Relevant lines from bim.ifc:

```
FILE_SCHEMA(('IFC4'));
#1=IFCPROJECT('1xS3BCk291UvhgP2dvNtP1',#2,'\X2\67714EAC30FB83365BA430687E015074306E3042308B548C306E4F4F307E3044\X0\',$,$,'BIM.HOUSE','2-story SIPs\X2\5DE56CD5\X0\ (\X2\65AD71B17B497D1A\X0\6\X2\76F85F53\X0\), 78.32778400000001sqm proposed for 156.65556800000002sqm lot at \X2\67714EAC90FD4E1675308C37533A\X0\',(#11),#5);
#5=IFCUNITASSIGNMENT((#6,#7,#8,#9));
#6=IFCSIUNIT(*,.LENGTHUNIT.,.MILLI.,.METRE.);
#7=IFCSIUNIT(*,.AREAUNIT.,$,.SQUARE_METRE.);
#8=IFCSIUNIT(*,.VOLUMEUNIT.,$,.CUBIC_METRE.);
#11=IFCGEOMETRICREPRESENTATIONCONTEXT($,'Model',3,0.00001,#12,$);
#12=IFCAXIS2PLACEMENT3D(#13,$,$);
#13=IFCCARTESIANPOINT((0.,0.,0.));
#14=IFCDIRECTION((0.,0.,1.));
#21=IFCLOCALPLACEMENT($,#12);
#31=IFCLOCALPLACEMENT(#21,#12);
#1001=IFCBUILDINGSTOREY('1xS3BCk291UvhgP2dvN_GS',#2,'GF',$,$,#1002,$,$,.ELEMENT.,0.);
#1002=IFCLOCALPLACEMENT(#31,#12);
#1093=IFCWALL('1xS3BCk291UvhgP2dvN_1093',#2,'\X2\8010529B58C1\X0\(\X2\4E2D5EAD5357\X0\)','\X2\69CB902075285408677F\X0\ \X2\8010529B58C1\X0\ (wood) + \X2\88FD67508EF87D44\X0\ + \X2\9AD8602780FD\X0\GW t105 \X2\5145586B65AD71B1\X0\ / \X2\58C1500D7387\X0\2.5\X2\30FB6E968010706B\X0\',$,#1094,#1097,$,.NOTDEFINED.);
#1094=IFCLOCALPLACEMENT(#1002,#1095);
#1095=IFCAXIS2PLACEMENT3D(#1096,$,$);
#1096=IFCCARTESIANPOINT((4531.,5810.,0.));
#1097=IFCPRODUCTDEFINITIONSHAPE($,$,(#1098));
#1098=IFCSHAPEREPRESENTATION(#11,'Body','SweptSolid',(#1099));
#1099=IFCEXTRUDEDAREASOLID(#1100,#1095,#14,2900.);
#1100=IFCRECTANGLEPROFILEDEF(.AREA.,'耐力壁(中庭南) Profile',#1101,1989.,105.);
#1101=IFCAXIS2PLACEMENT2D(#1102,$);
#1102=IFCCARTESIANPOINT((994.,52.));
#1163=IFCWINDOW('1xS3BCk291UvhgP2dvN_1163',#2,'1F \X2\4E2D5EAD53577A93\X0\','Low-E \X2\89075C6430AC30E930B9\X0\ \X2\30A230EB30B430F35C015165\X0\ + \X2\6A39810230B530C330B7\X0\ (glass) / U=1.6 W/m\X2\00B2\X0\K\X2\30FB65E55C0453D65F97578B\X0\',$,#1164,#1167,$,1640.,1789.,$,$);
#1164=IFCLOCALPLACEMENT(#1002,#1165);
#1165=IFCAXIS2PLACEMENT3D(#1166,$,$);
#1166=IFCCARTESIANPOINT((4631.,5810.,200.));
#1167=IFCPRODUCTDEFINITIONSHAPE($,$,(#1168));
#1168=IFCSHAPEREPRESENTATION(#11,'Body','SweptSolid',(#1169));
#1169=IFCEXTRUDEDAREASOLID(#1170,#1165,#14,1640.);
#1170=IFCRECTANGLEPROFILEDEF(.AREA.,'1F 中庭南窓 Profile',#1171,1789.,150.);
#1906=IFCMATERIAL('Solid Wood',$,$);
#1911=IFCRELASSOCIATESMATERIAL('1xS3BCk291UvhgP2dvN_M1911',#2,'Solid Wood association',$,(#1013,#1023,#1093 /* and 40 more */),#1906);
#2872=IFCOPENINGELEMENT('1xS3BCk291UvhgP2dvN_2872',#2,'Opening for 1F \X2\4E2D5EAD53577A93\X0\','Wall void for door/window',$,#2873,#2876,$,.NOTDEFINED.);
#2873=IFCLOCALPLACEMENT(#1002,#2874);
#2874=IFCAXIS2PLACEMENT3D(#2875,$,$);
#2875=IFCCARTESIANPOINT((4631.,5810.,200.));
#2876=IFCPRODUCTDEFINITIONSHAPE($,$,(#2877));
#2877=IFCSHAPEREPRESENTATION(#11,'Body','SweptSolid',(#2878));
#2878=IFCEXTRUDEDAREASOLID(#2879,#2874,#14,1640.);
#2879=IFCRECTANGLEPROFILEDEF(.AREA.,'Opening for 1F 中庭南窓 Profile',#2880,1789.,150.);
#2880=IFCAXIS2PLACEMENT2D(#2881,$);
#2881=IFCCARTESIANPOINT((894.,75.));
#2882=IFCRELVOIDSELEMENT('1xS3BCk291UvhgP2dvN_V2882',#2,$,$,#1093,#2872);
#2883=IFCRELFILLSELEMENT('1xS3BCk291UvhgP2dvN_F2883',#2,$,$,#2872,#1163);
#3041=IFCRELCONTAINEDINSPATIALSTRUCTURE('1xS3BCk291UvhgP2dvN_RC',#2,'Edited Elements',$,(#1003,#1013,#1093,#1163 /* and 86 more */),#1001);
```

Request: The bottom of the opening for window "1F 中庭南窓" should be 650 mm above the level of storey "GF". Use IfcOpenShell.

```python
import numpy as np
import ifcopenshell
import ifcopenshell.api.geometry
import ifcopenshell.geom
import ifcopenshell.util.element
import ifcopenshell.util.placement
import ifcopenshell.util.shape
import ifcopenshell.util.unit

model = ifcopenshell.open("bim.ifc")
unit_scale = ifcopenshell.util.unit.calculate_unit_scale(model)

window = model.by_id(1163)
opening = window.FillsVoids[0].RelatingOpeningElement
storey = ifcopenshell.util.element.get_container(window, ifc_class="IfcBuildingStorey")
level = ifcopenshell.util.placement.get_local_placement(storey.ObjectPlacement)[2, 3]

# The opening's origin need not be at the sill, so measure its lowest point.
shape = ifcopenshell.geom.create_shape(ifcopenshell.geom.settings(), opening)
bottom = ifcopenshell.util.shape.get_shape_bottom_elevation(shape, shape.geometry) / unit_scale
dz = level + 0.65 / unit_scale - bottom

shift = np.array([0.0, 0.0, dz])
# The window is not placed relative to its opening, so move both.
for product in (opening, window):
    matrix = ifcopenshell.util.placement.get_local_placement(product.ObjectPlacement)
    matrix[:3, 3] += shift
    ifcopenshell.api.geometry.edit_object_placement(model, product=product, matrix=matrix, is_si=False)

print(f"moved by {dz * unit_scale:+.3f} m")

model.write("bim-out.ifc")
```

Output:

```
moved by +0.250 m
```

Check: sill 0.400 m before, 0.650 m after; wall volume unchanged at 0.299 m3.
